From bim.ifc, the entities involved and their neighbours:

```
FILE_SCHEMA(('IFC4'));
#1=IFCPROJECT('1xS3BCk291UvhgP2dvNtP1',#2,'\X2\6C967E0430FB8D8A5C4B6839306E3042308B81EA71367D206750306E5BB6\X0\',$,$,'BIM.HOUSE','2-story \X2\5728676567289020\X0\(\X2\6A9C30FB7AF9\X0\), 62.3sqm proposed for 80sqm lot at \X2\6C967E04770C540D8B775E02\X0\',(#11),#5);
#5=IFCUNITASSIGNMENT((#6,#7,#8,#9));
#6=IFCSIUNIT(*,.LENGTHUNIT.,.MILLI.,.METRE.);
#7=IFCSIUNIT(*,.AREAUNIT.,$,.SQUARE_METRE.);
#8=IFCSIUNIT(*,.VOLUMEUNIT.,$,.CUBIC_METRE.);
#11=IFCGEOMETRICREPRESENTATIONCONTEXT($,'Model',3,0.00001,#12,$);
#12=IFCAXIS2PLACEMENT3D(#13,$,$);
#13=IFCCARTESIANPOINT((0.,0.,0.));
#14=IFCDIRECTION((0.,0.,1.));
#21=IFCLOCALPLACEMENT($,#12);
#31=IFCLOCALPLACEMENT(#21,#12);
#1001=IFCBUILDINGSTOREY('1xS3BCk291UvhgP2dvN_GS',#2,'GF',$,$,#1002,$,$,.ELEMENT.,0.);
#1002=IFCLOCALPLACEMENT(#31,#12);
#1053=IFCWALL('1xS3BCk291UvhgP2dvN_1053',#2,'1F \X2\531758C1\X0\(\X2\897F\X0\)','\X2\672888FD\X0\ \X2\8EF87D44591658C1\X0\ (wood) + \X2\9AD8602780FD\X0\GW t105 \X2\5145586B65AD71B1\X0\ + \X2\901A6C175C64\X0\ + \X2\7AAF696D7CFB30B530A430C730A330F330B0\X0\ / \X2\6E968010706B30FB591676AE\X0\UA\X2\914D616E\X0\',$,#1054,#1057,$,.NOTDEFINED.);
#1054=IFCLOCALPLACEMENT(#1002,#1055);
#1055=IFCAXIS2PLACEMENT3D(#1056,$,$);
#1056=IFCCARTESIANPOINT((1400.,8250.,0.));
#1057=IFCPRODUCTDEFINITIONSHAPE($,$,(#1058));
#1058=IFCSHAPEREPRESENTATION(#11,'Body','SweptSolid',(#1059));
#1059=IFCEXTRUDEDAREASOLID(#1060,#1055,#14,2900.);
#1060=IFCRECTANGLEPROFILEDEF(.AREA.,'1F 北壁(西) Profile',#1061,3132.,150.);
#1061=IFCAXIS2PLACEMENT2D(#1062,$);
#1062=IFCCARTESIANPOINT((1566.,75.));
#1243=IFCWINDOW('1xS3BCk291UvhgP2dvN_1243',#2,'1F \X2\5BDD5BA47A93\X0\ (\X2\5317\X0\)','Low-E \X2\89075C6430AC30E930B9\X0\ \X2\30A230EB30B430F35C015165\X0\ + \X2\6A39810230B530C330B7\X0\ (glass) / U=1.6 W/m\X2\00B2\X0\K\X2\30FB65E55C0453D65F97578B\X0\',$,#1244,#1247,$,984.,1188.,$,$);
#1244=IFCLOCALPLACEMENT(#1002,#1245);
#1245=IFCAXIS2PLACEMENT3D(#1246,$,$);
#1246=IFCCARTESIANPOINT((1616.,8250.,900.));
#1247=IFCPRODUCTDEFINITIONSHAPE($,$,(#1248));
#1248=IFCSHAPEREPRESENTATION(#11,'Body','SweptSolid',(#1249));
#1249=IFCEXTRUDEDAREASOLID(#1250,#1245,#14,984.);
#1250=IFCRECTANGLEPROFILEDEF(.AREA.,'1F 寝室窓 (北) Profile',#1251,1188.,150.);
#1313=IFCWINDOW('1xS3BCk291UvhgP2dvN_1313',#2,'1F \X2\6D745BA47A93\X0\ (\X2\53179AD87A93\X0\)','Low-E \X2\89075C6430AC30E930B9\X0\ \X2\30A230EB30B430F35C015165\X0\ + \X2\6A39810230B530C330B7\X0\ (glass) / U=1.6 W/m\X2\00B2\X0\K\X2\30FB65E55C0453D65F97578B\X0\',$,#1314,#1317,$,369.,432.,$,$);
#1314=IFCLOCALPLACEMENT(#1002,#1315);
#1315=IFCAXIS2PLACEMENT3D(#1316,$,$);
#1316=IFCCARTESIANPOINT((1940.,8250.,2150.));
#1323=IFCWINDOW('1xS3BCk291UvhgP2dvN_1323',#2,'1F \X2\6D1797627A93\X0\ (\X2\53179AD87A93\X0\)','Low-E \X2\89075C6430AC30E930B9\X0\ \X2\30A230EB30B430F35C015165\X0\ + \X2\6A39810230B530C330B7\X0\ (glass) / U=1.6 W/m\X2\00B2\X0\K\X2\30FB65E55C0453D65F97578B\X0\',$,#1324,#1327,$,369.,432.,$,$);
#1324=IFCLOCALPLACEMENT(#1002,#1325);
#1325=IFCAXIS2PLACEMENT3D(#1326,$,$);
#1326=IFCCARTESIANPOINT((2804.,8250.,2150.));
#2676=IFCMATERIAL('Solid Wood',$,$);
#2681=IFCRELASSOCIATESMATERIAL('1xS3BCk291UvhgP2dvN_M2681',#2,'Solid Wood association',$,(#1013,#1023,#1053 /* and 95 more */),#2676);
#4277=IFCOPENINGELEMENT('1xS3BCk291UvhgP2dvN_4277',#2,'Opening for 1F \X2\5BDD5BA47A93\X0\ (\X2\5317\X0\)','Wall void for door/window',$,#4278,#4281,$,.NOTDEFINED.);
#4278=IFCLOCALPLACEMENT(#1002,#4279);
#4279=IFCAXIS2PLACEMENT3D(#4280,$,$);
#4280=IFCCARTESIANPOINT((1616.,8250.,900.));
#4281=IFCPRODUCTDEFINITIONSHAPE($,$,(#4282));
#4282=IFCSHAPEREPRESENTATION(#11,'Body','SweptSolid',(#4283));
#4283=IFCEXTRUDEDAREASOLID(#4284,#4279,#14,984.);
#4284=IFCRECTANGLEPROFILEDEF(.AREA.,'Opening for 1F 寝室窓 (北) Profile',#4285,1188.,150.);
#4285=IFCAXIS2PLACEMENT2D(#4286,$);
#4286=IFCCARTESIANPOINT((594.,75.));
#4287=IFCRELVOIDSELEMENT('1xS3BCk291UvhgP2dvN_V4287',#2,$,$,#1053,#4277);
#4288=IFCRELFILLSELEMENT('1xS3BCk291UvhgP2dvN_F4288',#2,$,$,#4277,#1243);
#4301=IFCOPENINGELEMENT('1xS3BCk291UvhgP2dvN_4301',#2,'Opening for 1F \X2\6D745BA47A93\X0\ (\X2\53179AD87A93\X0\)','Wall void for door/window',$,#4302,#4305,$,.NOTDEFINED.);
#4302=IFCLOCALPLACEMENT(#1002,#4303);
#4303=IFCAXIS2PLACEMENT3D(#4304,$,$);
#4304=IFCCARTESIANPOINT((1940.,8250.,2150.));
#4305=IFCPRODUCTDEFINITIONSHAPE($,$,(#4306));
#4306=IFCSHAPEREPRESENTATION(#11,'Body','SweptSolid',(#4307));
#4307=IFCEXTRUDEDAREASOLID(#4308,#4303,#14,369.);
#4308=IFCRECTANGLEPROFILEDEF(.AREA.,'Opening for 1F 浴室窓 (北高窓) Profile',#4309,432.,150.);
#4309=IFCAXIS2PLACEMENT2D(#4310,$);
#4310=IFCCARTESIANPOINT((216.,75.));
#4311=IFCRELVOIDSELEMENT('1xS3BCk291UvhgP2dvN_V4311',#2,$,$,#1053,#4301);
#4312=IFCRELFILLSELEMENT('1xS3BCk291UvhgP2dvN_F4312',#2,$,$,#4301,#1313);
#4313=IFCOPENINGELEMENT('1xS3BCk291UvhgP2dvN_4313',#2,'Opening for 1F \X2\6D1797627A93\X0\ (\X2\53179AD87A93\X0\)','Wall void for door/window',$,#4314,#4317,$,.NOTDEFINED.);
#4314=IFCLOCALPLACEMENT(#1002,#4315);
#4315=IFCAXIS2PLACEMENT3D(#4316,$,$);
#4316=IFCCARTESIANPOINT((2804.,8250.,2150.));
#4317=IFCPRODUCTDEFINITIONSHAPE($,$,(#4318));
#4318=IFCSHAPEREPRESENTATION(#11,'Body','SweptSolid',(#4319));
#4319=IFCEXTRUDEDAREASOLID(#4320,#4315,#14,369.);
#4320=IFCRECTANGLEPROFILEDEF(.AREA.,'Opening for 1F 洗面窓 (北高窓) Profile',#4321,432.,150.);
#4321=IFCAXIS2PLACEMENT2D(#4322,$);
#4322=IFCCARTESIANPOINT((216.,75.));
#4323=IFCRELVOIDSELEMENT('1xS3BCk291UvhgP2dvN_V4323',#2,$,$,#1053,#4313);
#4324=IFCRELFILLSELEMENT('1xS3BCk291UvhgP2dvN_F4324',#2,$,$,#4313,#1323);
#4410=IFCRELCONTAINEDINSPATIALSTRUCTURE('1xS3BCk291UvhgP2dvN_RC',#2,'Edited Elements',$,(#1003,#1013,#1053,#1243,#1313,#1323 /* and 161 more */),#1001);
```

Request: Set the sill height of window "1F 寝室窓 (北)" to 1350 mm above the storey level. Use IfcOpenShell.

```python
import numpy as np
import ifcopenshell
import ifcopenshell.api.geometry
import ifcopenshell.geom
import ifcopenshell.util.element
import ifcopenshell.util.placement
import ifcopenshell.util.shape
import ifcopenshell.util.unit

model = ifcopenshell.open("bim.ifc")
unit_scale = ifcopenshell.util.unit.calculate_unit_scale(model)

window = model.by_guid("1xS3BCk291UvhgP2dvN_1243")
opening = window.FillsVoids[0].RelatingOpeningElement
storey = ifcopenshell.util.element.get_container(window, ifc_class="IfcBuildingStorey")
level = ifcopenshell.util.placement.get_local_placement(storey.ObjectPlacement)[2, 3]

# The opening's origin need not be at the sill, so measure its lowest point.
shape = ifcopenshell.geom.create_shape(ifcopenshell.geom.settings(), opening)
bottom = ifcopenshell.util.shape.get_shape_bottom_elevation(shape, shape.geometry) / unit_scale
dz = level + 1.35 / unit_scale - bottom

shift = np.array([0.0, 0.0, dz])
# The window is not placed relative to its opening, so move both.
for product in (opening, window):
    matrix = ifcopenshell.util.placement.get_local_placement(product.ObjectPlacement)
    matrix[:3, 3] += shift
    ifcopenshell.api.geometry.edit_object_placement(model, product=product, matrix=matrix, is_si=False)

print(f"moved by {dz * unit_scale:+.3f} m")

model.write("bim_rev.ifc")
```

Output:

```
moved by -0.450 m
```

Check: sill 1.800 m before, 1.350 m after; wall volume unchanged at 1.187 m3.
